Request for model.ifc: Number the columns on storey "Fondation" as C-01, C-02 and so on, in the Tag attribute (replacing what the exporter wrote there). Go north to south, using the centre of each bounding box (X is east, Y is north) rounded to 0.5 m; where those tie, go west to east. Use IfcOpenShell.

First a look at what the model holds.

```python
import ifcopenshell
import ifcopenshell.util.element
import ifcopenshell.util.placement

model = ifcopenshell.open("model.ifc")
print(model.schema)
storey = next(s for s in model.by_type("IfcBuildingStorey") if s.Name == "Fondation")
columns = [e for e in ifcopenshell.util.element.get_decomposition(storey) if e.is_a("IfcColumn")]
for e in sorted(columns, key=lambda e: e.id()):
    origin = ifcopenshell.util.placement.get_local_placement(e.ObjectPlacement)[:3, 3]
    print(e.id(), e.Tag, e.Name, origin.round(2) + 0.0, sep=" | ")
```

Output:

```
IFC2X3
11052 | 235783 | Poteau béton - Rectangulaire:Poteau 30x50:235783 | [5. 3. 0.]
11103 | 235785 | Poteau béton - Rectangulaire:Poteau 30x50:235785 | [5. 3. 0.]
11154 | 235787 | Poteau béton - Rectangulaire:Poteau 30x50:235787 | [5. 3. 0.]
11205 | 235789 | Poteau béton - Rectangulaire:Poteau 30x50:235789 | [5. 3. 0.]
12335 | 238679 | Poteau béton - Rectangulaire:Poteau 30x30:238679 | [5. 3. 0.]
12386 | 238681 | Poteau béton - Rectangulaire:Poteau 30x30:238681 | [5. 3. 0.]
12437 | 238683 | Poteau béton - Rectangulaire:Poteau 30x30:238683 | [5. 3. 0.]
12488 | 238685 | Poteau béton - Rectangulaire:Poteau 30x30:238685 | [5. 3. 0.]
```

```python
import ifcopenshell
import ifcopenshell.geom
import ifcopenshell.util.element
import ifcopenshell.util.shape

model = ifcopenshell.open("model.ifc")
settings = ifcopenshell.geom.settings()
settings.set("use-world-coords", True)


def centre(element):
    shape = ifcopenshell.geom.create_shape(settings, element)
    return ifcopenshell.util.shape.get_bbox_centroid(shape.geometry)


storey = next(s for s in model.by_type("IfcBuildingStorey") if s.Name == "Fondation")
columns = [e for e in ifcopenshell.util.element.get_decomposition(storey) if e.is_a("IfcColumn")]

# Insertion points can sit at a corner or the storey origin, so sort by the geometry (in metres).
centres = {e: centre(e) for e in columns}
columns.sort(key=lambda e: (-round(centres[e][1] / 0.5), centres[e][0]))

for i, e in enumerate(columns, start=1):
    number = f"C-{i:02d}"
    e.Tag = number
    print(e.id(), number)

model.write("model_updated.ifc")
```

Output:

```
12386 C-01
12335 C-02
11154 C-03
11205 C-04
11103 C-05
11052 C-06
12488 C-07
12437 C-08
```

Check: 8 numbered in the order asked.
